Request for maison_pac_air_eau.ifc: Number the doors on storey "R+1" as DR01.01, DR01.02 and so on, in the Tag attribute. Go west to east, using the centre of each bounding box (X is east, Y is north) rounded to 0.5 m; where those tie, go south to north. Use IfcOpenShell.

First a look at what the model holds.

```python
import ifcopenshell
import ifcopenshell.util.element
import ifcopenshell.util.placement

model = ifcopenshell.open("maison_pac_air_eau.ifc")
print(model.schema)
storey = next(s for s in model.by_type("IfcBuildingStorey") if s.Name == "R+1")
doors = [e for e in ifcopenshell.util.element.get_decomposition(storey) if e.is_a("IfcDoor")]
for e in sorted(doors, key=lambda e: e.id()):
    origin = ifcopenshell.util.placement.get_local_placement(e.ObjectPlacement)[:3, 3]
    print(e.id(), e.Tag, e.Name, origin.round(2) + 0.0, sep=" | ")
```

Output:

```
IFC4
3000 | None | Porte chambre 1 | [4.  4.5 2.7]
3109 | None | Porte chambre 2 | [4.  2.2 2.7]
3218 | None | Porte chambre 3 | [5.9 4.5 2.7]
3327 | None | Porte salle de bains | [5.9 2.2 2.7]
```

```python
import ifcopenshell
import ifcopenshell.geom
import ifcopenshell.util.element
import ifcopenshell.util.shape

model = ifcopenshell.open("maison_pac_air_eau.ifc")
settings = ifcopenshell.geom.settings()
settings.set("use-world-coords", True)


def centre(element):
    shape = ifcopenshell.geom.create_shape(settings, element)
    return ifcopenshell.util.shape.get_bbox_centroid(shape.geometry)


storey = next(s for s in model.by_type("IfcBuildingStorey") if s.Name == "R+1")
doors = [e for e in ifcopenshell.util.element.get_decomposition(storey) if e.is_a("IfcDoor")]

# Insertion points can sit at a corner or the storey origin, so sort by the geometry (in metres).
centres = {e: centre(e) for e in doors}
doors.sort(key=lambda e: (round(centres[e][0] / 0.5), centres[e][1]))

for i, e in enumerate(doors, start=1):
    number = f"DR01.{i:02d}"
    e.Tag = number
    print(e.id(), number)

model.write("maison_pac_air_eau_edited.ifc")
```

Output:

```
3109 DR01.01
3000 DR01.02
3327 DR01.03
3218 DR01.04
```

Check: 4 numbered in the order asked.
